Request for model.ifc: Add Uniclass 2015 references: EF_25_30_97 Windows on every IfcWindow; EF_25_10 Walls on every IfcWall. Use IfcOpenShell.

First a look at what the model holds.

```python
import ifcopenshell

model = ifcopenshell.open("model.ifc")
print(model.schema)
print("classifications:", [c.Name for c in model.by_type("IfcClassification")])
for ifc_class in ("IfcDoor", "IfcRoof", "IfcStair", "IfcWall", "IfcWindow"):
    print(ifc_class, len(model.by_type(ifc_class)))
```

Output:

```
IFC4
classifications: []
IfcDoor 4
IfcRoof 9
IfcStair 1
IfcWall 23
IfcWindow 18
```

```python
import ifcopenshell
import ifcopenshell.api.classification

model = ifcopenshell.open("model.ifc")

system = ifcopenshell.api.classification.add_classification(model, classification="Uniclass 2015")

codes = {
    "IfcWindow": ("EF_25_30_97", "Windows"),
    "IfcWall": ("EF_25_10", "Walls"),
}
for ifc_class, (code, name) in codes.items():
    products = model.by_type(ifc_class)
    ifcopenshell.api.classification.add_reference(
        model, products=products, classification=system, identification=code, name=name
    )
    print(code, len(products))

model.write("model_v2.ifc")
```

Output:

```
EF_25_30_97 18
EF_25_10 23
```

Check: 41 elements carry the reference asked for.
